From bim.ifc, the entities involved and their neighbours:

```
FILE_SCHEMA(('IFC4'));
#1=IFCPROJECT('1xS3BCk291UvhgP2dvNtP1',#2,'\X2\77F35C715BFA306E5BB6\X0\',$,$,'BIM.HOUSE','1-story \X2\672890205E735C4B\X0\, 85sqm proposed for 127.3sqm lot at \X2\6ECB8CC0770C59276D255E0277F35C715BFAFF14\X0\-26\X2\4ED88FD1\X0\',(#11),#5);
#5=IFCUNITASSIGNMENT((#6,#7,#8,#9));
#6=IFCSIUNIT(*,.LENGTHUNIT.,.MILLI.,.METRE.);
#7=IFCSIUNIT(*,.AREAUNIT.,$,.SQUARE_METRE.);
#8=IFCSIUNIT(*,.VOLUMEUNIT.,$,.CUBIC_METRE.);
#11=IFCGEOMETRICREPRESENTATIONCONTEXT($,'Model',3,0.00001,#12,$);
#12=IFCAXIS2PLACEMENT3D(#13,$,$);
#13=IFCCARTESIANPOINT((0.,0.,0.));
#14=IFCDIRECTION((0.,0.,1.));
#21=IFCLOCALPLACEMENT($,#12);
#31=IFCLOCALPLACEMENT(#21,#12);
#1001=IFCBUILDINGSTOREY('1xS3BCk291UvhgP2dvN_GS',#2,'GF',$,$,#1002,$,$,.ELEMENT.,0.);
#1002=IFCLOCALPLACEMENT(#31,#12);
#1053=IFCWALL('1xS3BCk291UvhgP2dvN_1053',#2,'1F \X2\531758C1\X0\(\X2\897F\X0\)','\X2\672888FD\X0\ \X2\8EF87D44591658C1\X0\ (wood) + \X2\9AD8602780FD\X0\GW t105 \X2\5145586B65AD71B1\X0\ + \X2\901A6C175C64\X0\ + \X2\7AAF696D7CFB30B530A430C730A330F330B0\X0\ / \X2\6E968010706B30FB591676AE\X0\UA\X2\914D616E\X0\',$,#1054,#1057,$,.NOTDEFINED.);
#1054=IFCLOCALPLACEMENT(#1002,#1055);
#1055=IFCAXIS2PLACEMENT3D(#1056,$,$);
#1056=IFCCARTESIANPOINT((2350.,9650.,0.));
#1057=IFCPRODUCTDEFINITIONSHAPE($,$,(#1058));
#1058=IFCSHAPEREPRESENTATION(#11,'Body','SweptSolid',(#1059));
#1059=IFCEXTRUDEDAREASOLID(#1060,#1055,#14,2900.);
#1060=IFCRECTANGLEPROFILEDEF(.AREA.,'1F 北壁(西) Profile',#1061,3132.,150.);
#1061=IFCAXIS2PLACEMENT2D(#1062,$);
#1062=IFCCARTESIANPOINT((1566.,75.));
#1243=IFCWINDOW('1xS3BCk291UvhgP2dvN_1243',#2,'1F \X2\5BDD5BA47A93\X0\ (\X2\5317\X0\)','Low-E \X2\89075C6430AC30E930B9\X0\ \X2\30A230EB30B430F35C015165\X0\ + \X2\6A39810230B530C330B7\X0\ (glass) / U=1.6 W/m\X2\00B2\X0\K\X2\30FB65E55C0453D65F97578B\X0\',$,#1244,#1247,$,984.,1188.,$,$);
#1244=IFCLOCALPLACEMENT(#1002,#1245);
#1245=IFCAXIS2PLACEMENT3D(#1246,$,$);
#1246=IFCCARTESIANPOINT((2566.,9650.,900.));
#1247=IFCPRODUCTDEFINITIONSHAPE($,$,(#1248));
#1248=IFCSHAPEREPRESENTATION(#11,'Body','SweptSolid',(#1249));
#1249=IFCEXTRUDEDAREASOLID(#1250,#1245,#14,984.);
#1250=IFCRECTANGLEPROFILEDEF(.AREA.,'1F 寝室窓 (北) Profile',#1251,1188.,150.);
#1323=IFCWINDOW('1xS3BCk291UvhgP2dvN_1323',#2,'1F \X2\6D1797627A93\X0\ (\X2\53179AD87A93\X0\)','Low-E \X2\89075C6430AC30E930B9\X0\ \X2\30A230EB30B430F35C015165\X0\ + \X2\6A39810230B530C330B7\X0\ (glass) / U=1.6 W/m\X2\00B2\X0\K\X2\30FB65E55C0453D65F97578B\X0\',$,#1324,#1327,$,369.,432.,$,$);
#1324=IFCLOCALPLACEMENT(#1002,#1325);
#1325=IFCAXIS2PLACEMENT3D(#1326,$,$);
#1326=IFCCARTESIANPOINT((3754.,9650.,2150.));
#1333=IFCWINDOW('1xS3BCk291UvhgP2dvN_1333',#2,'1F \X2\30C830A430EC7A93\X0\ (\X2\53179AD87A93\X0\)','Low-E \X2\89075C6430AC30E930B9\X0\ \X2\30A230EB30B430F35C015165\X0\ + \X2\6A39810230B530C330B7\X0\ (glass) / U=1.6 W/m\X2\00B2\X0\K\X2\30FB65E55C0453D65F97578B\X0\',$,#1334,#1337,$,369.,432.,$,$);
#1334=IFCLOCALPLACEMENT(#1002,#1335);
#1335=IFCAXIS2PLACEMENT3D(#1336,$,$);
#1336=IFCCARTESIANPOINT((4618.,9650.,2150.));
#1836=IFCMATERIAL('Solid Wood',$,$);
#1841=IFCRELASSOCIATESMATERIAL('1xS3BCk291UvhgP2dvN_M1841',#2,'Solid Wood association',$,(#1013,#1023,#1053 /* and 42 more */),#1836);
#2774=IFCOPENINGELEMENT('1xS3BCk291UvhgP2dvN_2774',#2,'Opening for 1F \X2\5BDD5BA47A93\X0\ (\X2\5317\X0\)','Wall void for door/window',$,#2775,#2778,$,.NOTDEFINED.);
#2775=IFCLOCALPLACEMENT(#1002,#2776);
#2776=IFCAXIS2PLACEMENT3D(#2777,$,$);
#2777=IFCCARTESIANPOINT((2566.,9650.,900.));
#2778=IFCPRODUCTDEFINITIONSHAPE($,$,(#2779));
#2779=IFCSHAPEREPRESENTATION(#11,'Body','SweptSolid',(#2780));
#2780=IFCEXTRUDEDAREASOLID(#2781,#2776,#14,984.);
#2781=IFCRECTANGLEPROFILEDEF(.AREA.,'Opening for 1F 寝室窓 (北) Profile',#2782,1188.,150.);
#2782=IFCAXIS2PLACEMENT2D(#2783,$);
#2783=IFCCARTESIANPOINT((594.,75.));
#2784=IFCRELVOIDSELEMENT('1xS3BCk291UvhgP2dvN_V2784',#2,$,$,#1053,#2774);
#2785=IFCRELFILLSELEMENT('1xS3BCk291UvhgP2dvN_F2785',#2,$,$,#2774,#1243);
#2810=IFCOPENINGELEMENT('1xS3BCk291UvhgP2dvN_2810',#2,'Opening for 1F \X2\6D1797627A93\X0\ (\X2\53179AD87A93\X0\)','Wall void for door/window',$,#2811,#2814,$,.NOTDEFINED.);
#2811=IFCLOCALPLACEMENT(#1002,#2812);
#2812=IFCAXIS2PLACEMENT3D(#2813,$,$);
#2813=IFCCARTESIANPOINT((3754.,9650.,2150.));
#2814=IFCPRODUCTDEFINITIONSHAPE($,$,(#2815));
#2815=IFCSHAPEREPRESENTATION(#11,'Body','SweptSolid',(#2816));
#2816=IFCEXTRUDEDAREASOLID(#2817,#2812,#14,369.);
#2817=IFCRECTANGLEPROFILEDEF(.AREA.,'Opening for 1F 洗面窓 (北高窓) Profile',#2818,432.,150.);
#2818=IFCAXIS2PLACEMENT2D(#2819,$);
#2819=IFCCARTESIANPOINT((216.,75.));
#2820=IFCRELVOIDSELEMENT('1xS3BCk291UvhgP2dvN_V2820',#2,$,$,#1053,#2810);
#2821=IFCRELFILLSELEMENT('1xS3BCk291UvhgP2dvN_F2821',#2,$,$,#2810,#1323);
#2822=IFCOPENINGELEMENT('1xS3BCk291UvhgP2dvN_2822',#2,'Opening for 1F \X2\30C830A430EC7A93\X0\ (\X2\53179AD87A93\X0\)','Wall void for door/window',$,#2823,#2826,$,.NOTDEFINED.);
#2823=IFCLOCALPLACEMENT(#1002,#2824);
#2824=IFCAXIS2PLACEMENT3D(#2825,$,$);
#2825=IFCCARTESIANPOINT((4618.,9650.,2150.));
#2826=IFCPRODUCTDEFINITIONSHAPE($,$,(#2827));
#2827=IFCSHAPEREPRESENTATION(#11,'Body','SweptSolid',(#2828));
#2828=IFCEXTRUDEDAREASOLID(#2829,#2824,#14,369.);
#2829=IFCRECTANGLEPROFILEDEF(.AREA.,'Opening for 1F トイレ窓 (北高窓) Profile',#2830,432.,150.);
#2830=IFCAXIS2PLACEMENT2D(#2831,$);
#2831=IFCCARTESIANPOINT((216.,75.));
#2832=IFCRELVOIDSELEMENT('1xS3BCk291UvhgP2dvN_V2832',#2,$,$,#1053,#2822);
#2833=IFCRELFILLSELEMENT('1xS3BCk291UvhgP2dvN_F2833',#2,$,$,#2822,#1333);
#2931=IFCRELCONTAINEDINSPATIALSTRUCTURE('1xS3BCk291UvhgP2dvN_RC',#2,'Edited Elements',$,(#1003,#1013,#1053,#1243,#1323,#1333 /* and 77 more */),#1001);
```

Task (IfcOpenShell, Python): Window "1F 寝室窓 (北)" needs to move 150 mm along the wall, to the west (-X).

```python
import ifcopenshell
import ifcopenshell.api.geometry
import ifcopenshell.util.placement
import ifcopenshell.util.unit

model = ifcopenshell.open("bim.ifc")
unit_scale = ifcopenshell.util.unit.calculate_unit_scale(model)

window = model.by_guid("1xS3BCk291UvhgP2dvN_1243")
opening = window.FillsVoids[0].RelatingOpeningElement
wall = opening.VoidsElements[0].RelatingBuildingElement

wall_matrix = ifcopenshell.util.placement.get_local_placement(wall.ObjectPlacement)
shift = wall_matrix[:3, 0] * -0.15 / unit_scale
before = ifcopenshell.util.placement.get_local_placement(window.ObjectPlacement)[:3, 3].copy()

# The window is not placed relative to its opening, so move both.
for product in (opening, window):
    matrix = ifcopenshell.util.placement.get_local_placement(product.ObjectPlacement)
    matrix[:3, 3] += shift
    ifcopenshell.api.geometry.edit_object_placement(model, product=product, matrix=matrix, is_si=False)

after = ifcopenshell.util.placement.get_local_placement(window.ObjectPlacement)[:3, 3]
print("window moved by", (after - before).round(3) + 0.0)

model.write("bim_v2.ifc")
```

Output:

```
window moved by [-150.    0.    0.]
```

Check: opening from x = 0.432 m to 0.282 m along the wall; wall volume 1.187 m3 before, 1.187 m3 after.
